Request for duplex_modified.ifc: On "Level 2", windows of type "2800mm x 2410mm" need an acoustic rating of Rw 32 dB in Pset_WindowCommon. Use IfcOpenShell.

First a look at what the model holds.

```python
import ifcopenshell
import ifcopenshell.util.element

model = ifcopenshell.open("duplex_modified.ifc")
print(model.schema)
storey = next(s for s in model.by_type("IfcBuildingStorey") if s.Name == "Level 2")
windows = [e for e in ifcopenshell.util.element.get_decomposition(storey) if e.is_a("IfcWindow")]
seen = {}
for e in windows:
    element_type = ifcopenshell.util.element.get_type(e)
    key = (element_type.Name if element_type != e and element_type else None, ifcopenshell.util.element.get_pset(e, "Pset_WindowCommon", "AcousticRating"))
    seen[key] = seen.get(key, 0) + 1
for (name, value), count in sorted(seen.items(), key=str):
    print(count, "x", name, "|", value)
```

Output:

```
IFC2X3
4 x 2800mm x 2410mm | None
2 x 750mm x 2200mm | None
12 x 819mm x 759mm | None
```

```python
import ifcopenshell
import ifcopenshell.api.pset
import ifcopenshell.util.element

model = ifcopenshell.open("duplex_modified.ifc")

storey = next(s for s in model.by_type("IfcBuildingStorey") if s.Name == "Level 2")
windows = [e for e in ifcopenshell.util.element.get_decomposition(storey) if e.is_a("IfcWindow")]

count = 0
for e in windows:
    element_type = ifcopenshell.util.element.get_type(e)
    if element_type in (None, e) or element_type.Name != "2800mm x 2410mm":
        continue
    # add_pset returns the element's existing set when there is one.
    pset = ifcopenshell.api.pset.add_pset(model, product=e, name="Pset_WindowCommon")
    ifcopenshell.api.pset.edit_pset(model, pset=pset, properties={"AcousticRating": "Rw 32 dB"})
    count += 1

print(count, "windows updated")

model.write("duplex_modified_v2.ifc")
```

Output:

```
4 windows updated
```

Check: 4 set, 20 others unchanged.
